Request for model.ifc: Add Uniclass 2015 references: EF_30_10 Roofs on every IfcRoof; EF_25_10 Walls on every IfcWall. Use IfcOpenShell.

First a look at what the model holds.

```python
import ifcopenshell

model = ifcopenshell.open("model.ifc")
print(model.schema)
print("classifications:", [c.Name for c in model.by_type("IfcClassification")])
for ifc_class in ("IfcDoor", "IfcRoof", "IfcStair", "IfcWall", "IfcWindow"):
    print(ifc_class, len(model.by_type(ifc_class)))
```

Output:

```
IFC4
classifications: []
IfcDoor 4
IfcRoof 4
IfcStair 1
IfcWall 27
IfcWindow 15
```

```python
import ifcopenshell
import ifcopenshell.api.classification

model = ifcopenshell.open("model.ifc")

system = ifcopenshell.api.classification.add_classification(model, classification="Uniclass 2015")

codes = {
    "IfcRoof": ("EF_30_10", "Roofs"),
    "IfcWall": ("EF_25_10", "Walls"),
}
for ifc_class, (code, name) in codes.items():
    products = model.by_type(ifc_class)
    ifcopenshell.api.classification.add_reference(
        model, products=products, classification=system, identification=code, name=name
    )
    print(code, len(products))

model.write("model_edited.ifc")
```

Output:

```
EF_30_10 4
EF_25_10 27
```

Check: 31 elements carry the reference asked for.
